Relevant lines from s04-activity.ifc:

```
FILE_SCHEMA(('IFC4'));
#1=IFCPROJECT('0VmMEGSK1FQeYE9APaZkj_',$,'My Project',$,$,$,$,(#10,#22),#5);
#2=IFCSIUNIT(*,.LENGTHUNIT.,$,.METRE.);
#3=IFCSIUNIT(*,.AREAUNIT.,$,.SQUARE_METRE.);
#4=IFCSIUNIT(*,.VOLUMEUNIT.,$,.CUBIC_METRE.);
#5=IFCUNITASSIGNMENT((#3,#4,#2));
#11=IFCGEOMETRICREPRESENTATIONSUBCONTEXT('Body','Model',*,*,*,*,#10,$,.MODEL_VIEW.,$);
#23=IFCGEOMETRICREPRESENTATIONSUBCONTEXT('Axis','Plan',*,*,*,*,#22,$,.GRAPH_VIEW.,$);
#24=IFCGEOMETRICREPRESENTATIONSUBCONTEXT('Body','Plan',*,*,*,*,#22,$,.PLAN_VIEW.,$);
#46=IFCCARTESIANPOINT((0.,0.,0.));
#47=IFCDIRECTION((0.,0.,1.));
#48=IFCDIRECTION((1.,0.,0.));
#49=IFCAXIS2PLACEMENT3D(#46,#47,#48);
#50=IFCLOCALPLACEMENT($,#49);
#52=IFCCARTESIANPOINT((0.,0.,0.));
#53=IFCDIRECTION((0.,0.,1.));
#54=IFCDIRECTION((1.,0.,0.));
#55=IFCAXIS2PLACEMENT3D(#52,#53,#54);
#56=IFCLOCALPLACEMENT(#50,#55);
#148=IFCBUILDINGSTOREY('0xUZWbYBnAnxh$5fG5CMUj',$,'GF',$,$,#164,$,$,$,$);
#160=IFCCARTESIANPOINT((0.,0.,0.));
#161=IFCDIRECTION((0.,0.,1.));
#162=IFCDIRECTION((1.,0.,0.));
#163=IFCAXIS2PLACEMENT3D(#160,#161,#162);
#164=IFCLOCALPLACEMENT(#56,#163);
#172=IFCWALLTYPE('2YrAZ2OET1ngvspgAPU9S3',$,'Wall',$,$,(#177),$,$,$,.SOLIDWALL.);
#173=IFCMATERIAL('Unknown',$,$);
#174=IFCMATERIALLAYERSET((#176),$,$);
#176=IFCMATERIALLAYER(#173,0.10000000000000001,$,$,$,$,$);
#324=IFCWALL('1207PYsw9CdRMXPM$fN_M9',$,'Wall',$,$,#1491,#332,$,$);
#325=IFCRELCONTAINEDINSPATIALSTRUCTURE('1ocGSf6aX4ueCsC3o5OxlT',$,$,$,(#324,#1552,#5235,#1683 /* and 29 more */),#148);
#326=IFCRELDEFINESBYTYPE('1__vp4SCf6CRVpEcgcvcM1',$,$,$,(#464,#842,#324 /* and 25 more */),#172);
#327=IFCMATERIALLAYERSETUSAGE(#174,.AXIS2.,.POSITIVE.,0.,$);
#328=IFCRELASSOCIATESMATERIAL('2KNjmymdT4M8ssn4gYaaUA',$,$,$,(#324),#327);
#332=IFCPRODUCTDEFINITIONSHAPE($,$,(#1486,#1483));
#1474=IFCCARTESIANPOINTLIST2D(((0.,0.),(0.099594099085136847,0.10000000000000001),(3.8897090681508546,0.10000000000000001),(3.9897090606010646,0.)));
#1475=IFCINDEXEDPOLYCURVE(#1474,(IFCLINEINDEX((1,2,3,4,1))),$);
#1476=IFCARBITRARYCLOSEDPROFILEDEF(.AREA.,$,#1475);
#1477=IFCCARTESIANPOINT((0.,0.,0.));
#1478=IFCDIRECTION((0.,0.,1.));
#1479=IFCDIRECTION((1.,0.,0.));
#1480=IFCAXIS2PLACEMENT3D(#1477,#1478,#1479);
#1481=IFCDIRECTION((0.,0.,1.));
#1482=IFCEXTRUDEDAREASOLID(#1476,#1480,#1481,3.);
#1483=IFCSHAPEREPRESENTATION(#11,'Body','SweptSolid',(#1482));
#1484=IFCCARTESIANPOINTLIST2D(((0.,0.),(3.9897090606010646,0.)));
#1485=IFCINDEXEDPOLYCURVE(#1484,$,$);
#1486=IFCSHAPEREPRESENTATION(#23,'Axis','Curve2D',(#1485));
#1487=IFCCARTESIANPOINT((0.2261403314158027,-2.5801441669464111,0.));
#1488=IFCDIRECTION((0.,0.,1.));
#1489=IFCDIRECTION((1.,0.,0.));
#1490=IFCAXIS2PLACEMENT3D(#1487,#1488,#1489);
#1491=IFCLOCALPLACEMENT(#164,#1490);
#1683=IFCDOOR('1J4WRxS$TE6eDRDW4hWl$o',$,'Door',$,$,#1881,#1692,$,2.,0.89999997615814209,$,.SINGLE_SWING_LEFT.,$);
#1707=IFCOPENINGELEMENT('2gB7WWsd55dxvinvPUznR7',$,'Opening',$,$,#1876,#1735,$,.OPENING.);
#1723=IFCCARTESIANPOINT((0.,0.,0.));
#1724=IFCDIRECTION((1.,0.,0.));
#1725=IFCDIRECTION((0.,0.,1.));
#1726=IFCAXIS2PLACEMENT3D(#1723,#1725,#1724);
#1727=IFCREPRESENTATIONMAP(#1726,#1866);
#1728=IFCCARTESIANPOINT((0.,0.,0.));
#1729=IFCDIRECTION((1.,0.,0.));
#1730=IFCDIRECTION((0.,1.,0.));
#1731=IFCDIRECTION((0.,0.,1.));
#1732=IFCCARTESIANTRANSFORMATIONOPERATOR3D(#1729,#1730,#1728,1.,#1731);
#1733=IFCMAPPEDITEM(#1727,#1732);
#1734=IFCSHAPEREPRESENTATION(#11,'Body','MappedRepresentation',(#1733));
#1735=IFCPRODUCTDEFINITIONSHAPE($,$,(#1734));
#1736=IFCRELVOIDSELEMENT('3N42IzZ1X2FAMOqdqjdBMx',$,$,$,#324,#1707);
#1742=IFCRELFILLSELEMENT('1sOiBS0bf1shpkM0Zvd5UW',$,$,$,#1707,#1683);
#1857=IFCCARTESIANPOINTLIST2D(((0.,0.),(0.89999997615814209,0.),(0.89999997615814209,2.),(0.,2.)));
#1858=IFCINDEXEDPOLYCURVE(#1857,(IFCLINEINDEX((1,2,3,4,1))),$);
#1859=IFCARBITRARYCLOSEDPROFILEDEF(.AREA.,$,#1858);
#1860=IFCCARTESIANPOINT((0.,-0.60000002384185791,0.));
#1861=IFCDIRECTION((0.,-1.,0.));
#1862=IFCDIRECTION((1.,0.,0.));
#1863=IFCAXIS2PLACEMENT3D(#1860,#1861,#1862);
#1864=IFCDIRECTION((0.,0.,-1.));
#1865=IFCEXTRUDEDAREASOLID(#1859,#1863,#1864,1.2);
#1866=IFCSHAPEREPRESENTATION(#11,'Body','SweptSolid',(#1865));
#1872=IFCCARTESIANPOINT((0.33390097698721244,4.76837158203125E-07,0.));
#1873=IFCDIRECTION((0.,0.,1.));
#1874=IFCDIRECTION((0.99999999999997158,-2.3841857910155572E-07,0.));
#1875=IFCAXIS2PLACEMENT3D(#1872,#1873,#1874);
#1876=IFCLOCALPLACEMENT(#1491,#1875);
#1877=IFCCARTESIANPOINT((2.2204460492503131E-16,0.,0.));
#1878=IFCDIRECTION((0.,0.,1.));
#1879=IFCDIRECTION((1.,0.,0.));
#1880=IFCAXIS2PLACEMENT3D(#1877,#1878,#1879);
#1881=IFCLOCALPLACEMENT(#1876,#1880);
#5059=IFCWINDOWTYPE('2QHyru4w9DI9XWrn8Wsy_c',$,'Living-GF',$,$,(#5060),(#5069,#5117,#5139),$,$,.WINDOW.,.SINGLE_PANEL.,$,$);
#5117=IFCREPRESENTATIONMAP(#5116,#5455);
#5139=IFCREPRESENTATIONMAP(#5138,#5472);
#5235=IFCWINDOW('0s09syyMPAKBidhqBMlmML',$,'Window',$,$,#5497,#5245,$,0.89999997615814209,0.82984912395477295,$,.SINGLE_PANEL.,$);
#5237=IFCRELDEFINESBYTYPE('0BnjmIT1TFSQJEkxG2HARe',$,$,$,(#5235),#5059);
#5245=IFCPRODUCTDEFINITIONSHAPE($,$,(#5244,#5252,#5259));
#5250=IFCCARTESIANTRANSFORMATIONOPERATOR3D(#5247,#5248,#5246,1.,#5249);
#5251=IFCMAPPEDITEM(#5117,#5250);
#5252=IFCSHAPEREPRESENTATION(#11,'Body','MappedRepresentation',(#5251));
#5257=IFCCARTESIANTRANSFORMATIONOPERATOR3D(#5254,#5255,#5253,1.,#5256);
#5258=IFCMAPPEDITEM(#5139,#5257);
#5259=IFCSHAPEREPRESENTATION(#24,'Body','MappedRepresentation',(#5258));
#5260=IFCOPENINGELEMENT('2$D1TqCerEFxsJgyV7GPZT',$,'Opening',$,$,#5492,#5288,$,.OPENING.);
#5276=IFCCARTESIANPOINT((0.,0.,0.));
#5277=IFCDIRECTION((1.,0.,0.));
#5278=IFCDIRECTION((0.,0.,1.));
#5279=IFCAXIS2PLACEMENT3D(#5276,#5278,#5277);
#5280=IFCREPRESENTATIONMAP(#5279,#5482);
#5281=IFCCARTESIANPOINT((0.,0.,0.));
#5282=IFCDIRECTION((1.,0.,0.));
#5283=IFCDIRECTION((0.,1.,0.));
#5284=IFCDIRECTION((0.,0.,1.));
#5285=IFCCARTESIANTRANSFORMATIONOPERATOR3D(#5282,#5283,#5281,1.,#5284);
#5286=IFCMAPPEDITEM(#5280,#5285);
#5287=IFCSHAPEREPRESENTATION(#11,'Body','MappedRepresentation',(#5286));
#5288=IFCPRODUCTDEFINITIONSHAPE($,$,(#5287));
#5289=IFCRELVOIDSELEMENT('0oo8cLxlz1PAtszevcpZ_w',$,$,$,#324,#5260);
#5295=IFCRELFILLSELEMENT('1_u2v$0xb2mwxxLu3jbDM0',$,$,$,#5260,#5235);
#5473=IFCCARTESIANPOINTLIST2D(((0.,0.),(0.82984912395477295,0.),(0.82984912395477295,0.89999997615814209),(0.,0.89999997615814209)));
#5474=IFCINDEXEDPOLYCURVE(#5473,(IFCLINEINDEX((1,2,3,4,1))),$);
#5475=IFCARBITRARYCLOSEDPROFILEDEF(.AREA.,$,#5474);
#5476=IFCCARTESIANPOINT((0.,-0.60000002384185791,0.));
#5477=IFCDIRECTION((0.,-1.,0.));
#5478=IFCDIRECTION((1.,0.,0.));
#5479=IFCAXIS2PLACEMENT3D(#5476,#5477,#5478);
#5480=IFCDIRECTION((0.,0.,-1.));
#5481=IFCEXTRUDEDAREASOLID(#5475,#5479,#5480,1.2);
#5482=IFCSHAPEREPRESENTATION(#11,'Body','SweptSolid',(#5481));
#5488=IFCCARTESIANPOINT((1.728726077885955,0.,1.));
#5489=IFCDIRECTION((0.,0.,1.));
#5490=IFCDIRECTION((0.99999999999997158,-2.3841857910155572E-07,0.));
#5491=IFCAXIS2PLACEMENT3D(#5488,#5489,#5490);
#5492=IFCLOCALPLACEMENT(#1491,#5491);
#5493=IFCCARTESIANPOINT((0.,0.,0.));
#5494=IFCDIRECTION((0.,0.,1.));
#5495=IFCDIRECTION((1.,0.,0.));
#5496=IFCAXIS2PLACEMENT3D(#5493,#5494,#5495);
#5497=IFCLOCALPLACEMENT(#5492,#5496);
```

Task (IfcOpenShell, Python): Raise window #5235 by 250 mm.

```python
import numpy as np
import ifcopenshell
import ifcopenshell.api.geometry
import ifcopenshell.util.placement
import ifcopenshell.util.unit

model = ifcopenshell.open("s04-activity.ifc")
unit_scale = ifcopenshell.util.unit.calculate_unit_scale(model)

window = model.by_guid("0s09syyMPAKBidhqBMlmML")
opening = window.FillsVoids[0].RelatingOpeningElement
dz = 0.25

shift = np.array([0.0, 0.0, dz])
# The window is placed relative to its opening, so it follows when the opening moves.
matrix = ifcopenshell.util.placement.get_local_placement(opening.ObjectPlacement)
matrix[:3, 3] += shift
ifcopenshell.api.geometry.edit_object_placement(
    model, product=opening, matrix=matrix, is_si=False, should_transform_children=True
)

print(f"moved by {dz * unit_scale:+.3f} m")

model.write("s04-activity_rev.ifc")
```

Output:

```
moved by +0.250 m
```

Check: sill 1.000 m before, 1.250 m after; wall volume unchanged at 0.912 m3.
